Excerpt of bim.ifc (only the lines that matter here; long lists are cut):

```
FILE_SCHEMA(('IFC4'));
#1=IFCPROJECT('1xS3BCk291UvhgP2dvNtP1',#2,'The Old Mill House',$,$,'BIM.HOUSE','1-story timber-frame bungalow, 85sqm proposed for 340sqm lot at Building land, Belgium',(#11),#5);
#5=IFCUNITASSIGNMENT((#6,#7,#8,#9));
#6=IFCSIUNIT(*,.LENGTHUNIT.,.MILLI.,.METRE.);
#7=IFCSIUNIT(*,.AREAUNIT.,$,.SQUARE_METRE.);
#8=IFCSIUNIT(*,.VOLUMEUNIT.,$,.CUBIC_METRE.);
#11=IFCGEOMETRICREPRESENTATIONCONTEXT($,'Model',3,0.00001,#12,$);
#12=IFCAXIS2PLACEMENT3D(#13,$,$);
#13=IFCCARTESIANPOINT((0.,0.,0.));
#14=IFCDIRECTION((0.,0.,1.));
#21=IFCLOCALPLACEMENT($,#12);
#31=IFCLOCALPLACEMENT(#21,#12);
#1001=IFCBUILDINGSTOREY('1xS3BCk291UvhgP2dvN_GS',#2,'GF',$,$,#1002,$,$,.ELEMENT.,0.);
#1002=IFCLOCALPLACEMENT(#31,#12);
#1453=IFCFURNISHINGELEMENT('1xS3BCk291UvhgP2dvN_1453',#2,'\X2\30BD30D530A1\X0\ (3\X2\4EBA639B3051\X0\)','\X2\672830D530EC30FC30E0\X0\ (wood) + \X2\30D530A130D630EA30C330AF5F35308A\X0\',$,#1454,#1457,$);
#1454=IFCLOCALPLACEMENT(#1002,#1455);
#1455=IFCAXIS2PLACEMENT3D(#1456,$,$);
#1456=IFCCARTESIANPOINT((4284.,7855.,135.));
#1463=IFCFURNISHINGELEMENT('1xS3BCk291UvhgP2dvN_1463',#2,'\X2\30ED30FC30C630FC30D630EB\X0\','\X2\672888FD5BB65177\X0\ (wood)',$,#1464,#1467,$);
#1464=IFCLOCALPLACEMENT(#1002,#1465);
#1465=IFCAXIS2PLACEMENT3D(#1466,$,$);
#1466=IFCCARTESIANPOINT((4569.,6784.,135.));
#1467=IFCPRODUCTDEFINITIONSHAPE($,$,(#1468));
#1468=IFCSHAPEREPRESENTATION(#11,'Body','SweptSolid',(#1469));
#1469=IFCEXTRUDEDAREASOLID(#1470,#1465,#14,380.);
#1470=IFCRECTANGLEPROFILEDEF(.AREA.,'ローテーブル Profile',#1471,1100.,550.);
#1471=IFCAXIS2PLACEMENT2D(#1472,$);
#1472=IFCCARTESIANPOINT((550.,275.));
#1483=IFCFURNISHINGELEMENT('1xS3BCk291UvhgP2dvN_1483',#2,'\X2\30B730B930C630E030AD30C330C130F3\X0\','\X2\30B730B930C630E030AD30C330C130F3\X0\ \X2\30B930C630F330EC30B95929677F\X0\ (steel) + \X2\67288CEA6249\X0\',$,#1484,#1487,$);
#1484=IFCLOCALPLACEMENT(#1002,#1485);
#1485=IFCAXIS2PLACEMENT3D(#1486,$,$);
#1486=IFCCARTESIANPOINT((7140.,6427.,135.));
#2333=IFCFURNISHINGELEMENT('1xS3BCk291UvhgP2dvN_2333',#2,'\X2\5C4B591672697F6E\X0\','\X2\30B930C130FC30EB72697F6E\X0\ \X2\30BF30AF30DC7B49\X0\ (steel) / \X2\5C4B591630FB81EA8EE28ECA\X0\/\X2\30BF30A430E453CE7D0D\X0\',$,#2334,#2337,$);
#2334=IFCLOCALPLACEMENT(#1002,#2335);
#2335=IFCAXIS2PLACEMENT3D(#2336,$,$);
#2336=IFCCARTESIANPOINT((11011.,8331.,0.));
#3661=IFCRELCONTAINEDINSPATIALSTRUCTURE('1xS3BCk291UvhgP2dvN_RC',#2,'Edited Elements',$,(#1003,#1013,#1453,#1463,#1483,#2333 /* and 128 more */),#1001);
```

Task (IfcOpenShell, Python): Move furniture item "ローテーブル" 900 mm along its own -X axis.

```python
import ifcopenshell
import ifcopenshell.api.geometry
import ifcopenshell.util.placement
import ifcopenshell.util.unit

model = ifcopenshell.open("bim.ifc")
unit_scale = ifcopenshell.util.unit.calculate_unit_scale(model)

item = model.by_guid("1xS3BCk291UvhgP2dvN_1463")
matrix = ifcopenshell.util.placement.get_local_placement(item.ObjectPlacement)
matrix[:3, 3] -= matrix[:3, 0] * 0.9 / unit_scale
ifcopenshell.api.geometry.edit_object_placement(model, product=item, matrix=matrix, is_si=False)

print(ifcopenshell.util.placement.get_local_placement(item.ObjectPlacement).round(3) + 0.0)

model.write("bim_v2.ifc")
```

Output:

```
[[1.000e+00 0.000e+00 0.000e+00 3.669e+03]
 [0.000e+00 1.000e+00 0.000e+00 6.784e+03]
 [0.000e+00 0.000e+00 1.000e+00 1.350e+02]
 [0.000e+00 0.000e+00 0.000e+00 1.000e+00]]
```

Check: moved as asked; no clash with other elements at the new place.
